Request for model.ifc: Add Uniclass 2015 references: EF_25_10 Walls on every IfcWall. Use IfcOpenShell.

First a look at what the model holds.

```python
import ifcopenshell

model = ifcopenshell.open("model.ifc")
print(model.schema)
print("classifications:", [c.Name for c in model.by_type("IfcClassification")])
for ifc_class in ("IfcDoor", "IfcRoof", "IfcStair", "IfcWall", "IfcWindow"):
    print(ifc_class, len(model.by_type(ifc_class)))
```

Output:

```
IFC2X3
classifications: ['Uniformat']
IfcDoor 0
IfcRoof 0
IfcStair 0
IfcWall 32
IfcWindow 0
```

```python
import ifcopenshell
import ifcopenshell.api.classification

model = ifcopenshell.open("model.ifc")

# IFC2X3 requires Source and Edition and has no link from the project to the system.
system = model.create_entity("IfcClassification", Source="NBS", Edition="2015", Name="Uniclass 2015")

codes = {
    "IfcWall": ("EF_25_10", "Walls"),
}
for ifc_class, (code, name) in codes.items():
    products = model.by_type(ifc_class)
    ifcopenshell.api.classification.add_reference(
        model, products=products, classification=system, identification=code, name=name
    )
    print(code, len(products))

model.write("model_updated.ifc")
```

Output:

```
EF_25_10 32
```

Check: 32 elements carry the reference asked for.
